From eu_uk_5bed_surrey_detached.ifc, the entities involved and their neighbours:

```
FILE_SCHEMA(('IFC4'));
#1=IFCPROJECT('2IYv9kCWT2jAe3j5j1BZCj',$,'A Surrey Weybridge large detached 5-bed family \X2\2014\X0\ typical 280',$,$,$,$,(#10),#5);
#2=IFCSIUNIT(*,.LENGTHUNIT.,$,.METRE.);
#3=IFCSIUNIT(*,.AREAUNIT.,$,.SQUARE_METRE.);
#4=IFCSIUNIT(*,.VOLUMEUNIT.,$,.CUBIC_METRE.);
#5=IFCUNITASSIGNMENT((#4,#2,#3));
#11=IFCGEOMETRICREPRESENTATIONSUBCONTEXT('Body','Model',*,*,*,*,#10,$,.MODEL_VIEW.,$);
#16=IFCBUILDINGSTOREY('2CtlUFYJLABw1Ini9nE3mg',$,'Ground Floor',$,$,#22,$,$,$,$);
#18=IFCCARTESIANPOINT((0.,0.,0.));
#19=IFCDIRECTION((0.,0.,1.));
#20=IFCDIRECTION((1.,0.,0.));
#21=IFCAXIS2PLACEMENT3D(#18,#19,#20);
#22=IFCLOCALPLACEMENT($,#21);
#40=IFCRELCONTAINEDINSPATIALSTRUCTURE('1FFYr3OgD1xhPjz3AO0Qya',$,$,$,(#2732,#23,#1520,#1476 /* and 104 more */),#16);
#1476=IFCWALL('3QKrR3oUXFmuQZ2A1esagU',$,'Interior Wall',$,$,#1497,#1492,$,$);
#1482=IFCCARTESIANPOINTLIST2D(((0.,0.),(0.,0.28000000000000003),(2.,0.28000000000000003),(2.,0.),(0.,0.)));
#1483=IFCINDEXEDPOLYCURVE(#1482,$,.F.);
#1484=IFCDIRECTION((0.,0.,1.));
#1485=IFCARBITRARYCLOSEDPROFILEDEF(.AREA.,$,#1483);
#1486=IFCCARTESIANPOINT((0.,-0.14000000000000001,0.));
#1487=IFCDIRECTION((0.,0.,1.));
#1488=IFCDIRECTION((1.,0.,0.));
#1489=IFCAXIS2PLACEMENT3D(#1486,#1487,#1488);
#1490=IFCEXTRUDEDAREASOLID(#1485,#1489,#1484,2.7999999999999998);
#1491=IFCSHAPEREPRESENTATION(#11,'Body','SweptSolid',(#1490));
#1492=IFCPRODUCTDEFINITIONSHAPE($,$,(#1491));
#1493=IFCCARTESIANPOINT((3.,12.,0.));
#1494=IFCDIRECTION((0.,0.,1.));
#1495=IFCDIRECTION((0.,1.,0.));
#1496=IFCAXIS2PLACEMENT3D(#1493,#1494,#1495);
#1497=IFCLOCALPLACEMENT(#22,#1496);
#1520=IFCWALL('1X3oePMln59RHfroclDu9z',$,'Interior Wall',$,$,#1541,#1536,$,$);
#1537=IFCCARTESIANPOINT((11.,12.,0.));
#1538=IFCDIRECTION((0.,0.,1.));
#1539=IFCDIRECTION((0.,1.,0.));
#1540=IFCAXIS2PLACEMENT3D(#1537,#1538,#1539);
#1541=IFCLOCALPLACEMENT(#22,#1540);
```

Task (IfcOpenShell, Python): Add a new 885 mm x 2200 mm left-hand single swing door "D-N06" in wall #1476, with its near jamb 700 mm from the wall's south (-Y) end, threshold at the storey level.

```python
import numpy as np
import ifcopenshell
import ifcopenshell.api.feature
import ifcopenshell.api.geometry
import ifcopenshell.api.root
import ifcopenshell.api.spatial
import ifcopenshell.geom
import ifcopenshell.util.element
import ifcopenshell.util.placement
import ifcopenshell.util.representation
import ifcopenshell.util.shape
import ifcopenshell.util.unit

model = ifcopenshell.open("eu_uk_5bed_surrey_detached.ifc")
unit_scale = ifcopenshell.util.unit.calculate_unit_scale(model)
settings = ifcopenshell.geom.settings()


def volume(element):
    """Net volume in cubic metres, openings subtracted."""
    shape = ifcopenshell.geom.create_shape(settings, element)
    return ifcopenshell.util.shape.get_volume(shape.geometry)


wall = model.by_guid("3QKrR3oUXFmuQZ2A1esagU")
storey = ifcopenshell.util.element.get_container(wall, ifc_class="IfcBuildingStorey")
context = ifcopenshell.util.representation.get_context(model, "Model", "Body", "MODEL_VIEW")
before = volume(wall)

width, height, from_end, sill = 0.885, 2.2, 0.7, 0.0  # metres

# The wall runs along its own X axis, and the end named is its -X end.
wall_shape = ifcopenshell.geom.create_shape(settings, wall)
x, y, z = ifcopenshell.util.shape.get_vertices(wall_shape.geometry).T
start = x.min() + from_end
face, thickness = float(y.min()), float(y.max() - y.min())
wall_matrix = ifcopenshell.util.placement.get_local_placement(wall.ObjectPlacement)
level = ifcopenshell.util.placement.get_local_placement(storey.ObjectPlacement)[2, 3]


def in_wall(x, y):
    """Placement at x, y metres in the wall's axes, at sill height."""
    matrix = wall_matrix.copy()
    matrix[:, 3] = wall_matrix @ np.array([x / unit_scale, y / unit_scale, 0.0, 1.0])
    matrix[2, 3] = level + sill / unit_scale
    return matrix


# Opening: a box that overshoots both wall faces by 50 mm.
opening = ifcopenshell.api.root.create_entity(model, ifc_class="IfcOpeningElement", predefined_type="OPENING")
box = ifcopenshell.api.geometry.add_wall_representation(
    model, context=context, length=width, height=height, thickness=thickness + 0.1
)
ifcopenshell.api.geometry.assign_representation(model, product=opening, representation=box)
ifcopenshell.api.geometry.edit_object_placement(model, product=opening, matrix=in_wall(start, face - 0.05), is_si=False)
ifcopenshell.api.feature.add_feature(model, feature=opening, element=wall)

door = ifcopenshell.api.root.create_entity(model, ifc_class="IfcDoor", name="D-N06", predefined_type="DOOR")
door.OverallWidth, door.OverallHeight = width / unit_scale, height / unit_scale
door.OperationType = "SINGLE_SWING_LEFT"
body = ifcopenshell.api.geometry.add_door_representation(
    model,
    context=context,
    overall_width=door.OverallWidth,
    overall_height=door.OverallHeight,
    operation_type="SINGLE_SWING_LEFT",
    lining_properties={"LiningDepth": thickness / unit_scale, "ThresholdDepth": thickness / unit_scale},
)
ifcopenshell.api.geometry.assign_representation(model, product=door, representation=body)
ifcopenshell.api.spatial.assign_container(model, products=[door], relating_structure=storey)
ifcopenshell.api.feature.add_filling(model, opening=opening, element=door)

# The lining spans the wall, so the door starts at the wall face.
ifcopenshell.api.geometry.edit_object_placement(model, product=door, matrix=in_wall(start, face), is_si=False)

after = volume(wall)

print(f"wall volume {before:.3f} -> {after:.3f} m3")

model.write("eu_uk_5bed_surrey_detached-out.ifc")
```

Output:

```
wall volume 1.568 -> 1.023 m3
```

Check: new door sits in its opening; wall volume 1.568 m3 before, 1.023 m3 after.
